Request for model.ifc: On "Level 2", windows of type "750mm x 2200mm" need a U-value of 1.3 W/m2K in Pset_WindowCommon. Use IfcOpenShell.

First a look at what the model holds.

```python
import ifcopenshell
import ifcopenshell.util.element

model = ifcopenshell.open("model.ifc")
print(model.schema)
storey = next(s for s in model.by_type("IfcBuildingStorey") if s.Name == "Level 2")
windows = [e for e in ifcopenshell.util.element.get_decomposition(storey) if e.is_a("IfcWindow")]
seen = {}
for e in windows:
    element_type = ifcopenshell.util.element.get_type(e)
    key = (element_type.Name if element_type != e and element_type else None, ifcopenshell.util.element.get_pset(e, "Pset_WindowCommon", "ThermalTransmittance"))
    seen[key] = seen.get(key, 0) + 1
for (name, value), count in sorted(seen.items(), key=str):
    print(count, "x", name, "|", value)
```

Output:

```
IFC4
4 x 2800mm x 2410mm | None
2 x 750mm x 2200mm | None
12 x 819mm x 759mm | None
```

```python
import ifcopenshell
import ifcopenshell.api.pset
import ifcopenshell.util.element

model = ifcopenshell.open("model.ifc")

storey = next(s for s in model.by_type("IfcBuildingStorey") if s.Name == "Level 2")
windows = [e for e in ifcopenshell.util.element.get_decomposition(storey) if e.is_a("IfcWindow")]

count = 0
for e in windows:
    element_type = ifcopenshell.util.element.get_type(e)
    if element_type in (None, e) or element_type.Name != "750mm x 2200mm":
        continue
    # add_pset returns the element's existing set when there is one.
    pset = ifcopenshell.api.pset.add_pset(model, product=e, name="Pset_WindowCommon")
    ifcopenshell.api.pset.edit_pset(model, pset=pset, properties={"ThermalTransmittance": 1.3})
    count += 1

print(count, "windows updated")

model.write("model_v2.ifc")
```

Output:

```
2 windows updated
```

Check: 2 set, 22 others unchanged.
